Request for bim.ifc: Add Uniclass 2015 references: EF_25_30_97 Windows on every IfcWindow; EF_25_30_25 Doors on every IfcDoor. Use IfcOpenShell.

First a look at what the model holds.

```python
import ifcopenshell

model = ifcopenshell.open("bim.ifc")
print(model.schema)
print("classifications:", [c.Name for c in model.by_type("IfcClassification")])
for ifc_class in ("IfcDoor", "IfcRoof", "IfcStair", "IfcWall", "IfcWindow"):
    print(ifc_class, len(model.by_type(ifc_class)))
```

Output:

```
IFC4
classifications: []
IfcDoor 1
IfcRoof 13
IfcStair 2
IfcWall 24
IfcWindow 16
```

```python
import ifcopenshell
import ifcopenshell.api.classification

model = ifcopenshell.open("bim.ifc")

system = ifcopenshell.api.classification.add_classification(model, classification="Uniclass 2015")

codes = {
    "IfcWindow": ("EF_25_30_97", "Windows"),
    "IfcDoor": ("EF_25_30_25", "Doors"),
}
for ifc_class, (code, name) in codes.items():
    products = model.by_type(ifc_class)
    ifcopenshell.api.classification.add_reference(
        model, products=products, classification=system, identification=code, name=name
    )
    print(code, len(products))

model.write("bim_updated.ifc")
```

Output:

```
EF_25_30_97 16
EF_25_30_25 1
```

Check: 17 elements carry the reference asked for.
